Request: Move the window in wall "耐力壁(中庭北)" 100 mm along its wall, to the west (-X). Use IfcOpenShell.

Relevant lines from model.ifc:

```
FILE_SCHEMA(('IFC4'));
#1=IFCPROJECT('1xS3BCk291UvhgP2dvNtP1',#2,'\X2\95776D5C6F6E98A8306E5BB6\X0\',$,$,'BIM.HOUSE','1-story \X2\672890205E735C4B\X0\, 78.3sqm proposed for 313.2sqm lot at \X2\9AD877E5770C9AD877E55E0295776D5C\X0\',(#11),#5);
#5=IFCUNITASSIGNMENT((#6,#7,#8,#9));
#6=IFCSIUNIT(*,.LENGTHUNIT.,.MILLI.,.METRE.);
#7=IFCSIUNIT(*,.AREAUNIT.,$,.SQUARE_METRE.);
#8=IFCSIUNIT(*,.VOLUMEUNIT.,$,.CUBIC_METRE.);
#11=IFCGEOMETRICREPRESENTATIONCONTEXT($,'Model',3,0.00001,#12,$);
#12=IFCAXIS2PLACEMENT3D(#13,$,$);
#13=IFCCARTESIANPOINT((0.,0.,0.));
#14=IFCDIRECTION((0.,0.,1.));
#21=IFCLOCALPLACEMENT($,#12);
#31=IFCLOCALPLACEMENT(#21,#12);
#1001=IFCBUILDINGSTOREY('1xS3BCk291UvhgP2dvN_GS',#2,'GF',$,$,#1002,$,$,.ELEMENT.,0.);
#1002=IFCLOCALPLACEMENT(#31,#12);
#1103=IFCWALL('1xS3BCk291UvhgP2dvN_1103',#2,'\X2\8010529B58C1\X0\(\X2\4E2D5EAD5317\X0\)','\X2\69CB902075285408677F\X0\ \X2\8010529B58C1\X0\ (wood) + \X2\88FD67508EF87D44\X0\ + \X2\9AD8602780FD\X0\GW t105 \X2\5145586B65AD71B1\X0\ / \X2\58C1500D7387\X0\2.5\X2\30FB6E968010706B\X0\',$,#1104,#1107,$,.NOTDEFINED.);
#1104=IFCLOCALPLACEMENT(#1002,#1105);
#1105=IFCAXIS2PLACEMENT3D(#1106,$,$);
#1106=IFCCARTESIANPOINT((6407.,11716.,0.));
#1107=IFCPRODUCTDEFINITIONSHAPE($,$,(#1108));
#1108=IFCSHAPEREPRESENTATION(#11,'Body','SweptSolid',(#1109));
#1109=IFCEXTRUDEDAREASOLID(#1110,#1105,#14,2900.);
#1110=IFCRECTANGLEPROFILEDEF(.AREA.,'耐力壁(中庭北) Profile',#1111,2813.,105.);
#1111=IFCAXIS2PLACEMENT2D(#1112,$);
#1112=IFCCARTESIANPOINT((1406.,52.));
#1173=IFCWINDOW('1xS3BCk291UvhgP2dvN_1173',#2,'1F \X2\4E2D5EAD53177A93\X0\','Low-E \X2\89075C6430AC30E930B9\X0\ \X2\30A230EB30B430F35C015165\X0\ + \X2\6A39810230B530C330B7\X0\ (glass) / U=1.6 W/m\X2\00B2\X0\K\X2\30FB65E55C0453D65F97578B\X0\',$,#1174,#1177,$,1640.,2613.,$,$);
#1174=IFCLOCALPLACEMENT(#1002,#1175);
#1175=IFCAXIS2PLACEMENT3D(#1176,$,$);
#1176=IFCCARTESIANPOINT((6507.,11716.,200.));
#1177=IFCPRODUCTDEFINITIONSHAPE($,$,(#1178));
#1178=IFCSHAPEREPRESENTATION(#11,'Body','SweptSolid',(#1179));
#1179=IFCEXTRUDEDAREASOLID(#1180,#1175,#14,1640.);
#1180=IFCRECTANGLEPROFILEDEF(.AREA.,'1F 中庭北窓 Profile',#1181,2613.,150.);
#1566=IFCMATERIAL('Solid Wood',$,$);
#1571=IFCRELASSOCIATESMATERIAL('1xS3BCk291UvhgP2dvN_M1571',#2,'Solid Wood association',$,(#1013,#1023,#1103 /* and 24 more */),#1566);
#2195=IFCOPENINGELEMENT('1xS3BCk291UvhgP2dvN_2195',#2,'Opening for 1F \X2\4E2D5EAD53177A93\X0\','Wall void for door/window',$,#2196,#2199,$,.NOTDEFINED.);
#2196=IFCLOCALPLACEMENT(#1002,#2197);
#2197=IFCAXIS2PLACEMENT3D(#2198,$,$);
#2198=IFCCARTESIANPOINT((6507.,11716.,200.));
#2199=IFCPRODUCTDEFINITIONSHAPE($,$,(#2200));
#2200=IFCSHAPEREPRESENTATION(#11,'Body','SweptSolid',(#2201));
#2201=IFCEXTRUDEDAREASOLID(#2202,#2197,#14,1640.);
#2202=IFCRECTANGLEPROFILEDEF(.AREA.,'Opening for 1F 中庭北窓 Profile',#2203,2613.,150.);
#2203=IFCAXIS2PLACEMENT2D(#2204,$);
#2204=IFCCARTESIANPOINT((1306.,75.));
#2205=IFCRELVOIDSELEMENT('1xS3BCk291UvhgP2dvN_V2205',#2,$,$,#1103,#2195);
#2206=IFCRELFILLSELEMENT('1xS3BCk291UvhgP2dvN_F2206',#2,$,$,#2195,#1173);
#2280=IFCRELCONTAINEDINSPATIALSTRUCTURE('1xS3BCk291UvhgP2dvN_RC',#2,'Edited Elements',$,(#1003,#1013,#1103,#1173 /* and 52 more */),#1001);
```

```python
import ifcopenshell
import ifcopenshell.api.geometry
import ifcopenshell.util.placement
import ifcopenshell.util.unit

model = ifcopenshell.open("model.ifc")
unit_scale = ifcopenshell.util.unit.calculate_unit_scale(model)

window = model.by_guid("1xS3BCk291UvhgP2dvN_1173")
opening = window.FillsVoids[0].RelatingOpeningElement
wall = opening.VoidsElements[0].RelatingBuildingElement

wall_matrix = ifcopenshell.util.placement.get_local_placement(wall.ObjectPlacement)
shift = wall_matrix[:3, 0] * -0.1 / unit_scale
before = ifcopenshell.util.placement.get_local_placement(window.ObjectPlacement)[:3, 3].copy()

# The window is not placed relative to its opening, so move both.
for product in (opening, window):
    matrix = ifcopenshell.util.placement.get_local_placement(product.ObjectPlacement)
    matrix[:3, 3] += shift
    ifcopenshell.api.geometry.edit_object_placement(model, product=product, matrix=matrix, is_si=False)

after = ifcopenshell.util.placement.get_local_placement(window.ObjectPlacement)[:3, 3]
print("window moved by", (after - before).round(3) + 0.0)

model.write("model_updated.ifc")
```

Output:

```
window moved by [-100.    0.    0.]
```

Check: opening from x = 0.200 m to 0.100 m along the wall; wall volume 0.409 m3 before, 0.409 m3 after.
